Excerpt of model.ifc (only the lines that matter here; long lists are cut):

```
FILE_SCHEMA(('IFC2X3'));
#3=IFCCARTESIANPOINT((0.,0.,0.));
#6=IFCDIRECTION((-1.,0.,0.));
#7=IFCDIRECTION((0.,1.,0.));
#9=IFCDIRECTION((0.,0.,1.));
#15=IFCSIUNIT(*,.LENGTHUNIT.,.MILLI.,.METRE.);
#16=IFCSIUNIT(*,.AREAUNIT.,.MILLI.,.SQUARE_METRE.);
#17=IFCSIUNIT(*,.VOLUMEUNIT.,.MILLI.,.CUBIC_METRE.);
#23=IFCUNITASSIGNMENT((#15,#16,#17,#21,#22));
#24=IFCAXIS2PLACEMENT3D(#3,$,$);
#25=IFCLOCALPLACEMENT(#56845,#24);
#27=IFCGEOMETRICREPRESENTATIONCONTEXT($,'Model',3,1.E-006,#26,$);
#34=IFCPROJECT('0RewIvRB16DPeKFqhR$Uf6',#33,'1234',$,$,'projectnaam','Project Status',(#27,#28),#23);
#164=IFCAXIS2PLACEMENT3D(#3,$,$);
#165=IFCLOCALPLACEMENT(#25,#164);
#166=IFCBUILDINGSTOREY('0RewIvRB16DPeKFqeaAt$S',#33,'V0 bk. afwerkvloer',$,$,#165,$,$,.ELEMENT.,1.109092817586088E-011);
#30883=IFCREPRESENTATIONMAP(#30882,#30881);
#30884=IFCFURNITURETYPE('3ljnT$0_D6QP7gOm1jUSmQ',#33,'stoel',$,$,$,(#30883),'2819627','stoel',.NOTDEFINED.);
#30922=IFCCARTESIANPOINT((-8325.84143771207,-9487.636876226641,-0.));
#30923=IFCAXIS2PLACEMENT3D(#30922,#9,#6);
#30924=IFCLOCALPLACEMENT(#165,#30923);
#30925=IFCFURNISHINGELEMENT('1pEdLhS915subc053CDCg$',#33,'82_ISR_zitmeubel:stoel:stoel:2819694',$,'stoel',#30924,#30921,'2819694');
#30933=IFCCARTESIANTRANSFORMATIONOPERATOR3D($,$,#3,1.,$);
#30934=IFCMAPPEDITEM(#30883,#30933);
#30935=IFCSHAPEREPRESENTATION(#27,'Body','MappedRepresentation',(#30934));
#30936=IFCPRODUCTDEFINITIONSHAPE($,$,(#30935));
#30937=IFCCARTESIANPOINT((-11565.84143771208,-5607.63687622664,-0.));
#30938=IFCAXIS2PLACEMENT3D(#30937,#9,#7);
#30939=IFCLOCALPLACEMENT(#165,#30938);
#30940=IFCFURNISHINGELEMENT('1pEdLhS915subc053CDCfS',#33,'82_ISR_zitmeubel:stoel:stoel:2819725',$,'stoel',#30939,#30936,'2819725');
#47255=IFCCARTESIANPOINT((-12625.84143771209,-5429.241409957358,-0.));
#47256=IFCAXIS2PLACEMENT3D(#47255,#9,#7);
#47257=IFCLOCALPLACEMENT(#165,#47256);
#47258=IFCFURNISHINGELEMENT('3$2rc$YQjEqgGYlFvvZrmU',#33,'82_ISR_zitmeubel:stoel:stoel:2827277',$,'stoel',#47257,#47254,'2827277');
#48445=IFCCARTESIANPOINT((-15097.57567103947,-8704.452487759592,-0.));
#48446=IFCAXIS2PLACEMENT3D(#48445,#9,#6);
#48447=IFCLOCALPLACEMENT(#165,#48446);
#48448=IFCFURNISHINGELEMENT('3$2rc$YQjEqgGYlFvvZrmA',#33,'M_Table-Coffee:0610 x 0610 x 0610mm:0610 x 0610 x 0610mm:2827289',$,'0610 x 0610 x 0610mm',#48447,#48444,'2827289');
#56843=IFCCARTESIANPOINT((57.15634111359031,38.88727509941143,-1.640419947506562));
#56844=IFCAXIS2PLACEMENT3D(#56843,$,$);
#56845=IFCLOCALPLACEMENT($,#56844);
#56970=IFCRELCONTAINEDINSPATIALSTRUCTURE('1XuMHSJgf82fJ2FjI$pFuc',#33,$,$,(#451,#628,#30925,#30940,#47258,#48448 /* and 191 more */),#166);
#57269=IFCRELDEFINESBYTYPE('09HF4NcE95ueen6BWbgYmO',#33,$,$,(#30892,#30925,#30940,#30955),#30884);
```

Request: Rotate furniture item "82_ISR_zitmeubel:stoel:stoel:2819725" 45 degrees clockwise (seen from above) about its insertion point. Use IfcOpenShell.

```python
import ifcopenshell
import ifcopenshell.api.geometry
import ifcopenshell.util.placement

model = ifcopenshell.open("model.ifc")

item = model.by_guid("1pEdLhS915subc053CDCfS")
matrix = ifcopenshell.util.placement.get_local_placement(item.ObjectPlacement)
matrix = matrix @ ifcopenshell.util.placement.rotation(-45, "Z")
ifcopenshell.api.geometry.edit_object_placement(model, product=item, matrix=matrix, is_si=False)

print(ifcopenshell.util.placement.get_local_placement(item.ObjectPlacement).round(3) + 0.0)

model.write("model_edited.ifc")
```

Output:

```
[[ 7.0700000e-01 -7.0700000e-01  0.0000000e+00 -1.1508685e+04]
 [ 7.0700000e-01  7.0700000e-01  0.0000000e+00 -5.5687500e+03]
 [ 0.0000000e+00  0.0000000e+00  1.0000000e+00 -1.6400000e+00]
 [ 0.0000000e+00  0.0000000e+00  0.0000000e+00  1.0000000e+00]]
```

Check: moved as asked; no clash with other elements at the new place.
